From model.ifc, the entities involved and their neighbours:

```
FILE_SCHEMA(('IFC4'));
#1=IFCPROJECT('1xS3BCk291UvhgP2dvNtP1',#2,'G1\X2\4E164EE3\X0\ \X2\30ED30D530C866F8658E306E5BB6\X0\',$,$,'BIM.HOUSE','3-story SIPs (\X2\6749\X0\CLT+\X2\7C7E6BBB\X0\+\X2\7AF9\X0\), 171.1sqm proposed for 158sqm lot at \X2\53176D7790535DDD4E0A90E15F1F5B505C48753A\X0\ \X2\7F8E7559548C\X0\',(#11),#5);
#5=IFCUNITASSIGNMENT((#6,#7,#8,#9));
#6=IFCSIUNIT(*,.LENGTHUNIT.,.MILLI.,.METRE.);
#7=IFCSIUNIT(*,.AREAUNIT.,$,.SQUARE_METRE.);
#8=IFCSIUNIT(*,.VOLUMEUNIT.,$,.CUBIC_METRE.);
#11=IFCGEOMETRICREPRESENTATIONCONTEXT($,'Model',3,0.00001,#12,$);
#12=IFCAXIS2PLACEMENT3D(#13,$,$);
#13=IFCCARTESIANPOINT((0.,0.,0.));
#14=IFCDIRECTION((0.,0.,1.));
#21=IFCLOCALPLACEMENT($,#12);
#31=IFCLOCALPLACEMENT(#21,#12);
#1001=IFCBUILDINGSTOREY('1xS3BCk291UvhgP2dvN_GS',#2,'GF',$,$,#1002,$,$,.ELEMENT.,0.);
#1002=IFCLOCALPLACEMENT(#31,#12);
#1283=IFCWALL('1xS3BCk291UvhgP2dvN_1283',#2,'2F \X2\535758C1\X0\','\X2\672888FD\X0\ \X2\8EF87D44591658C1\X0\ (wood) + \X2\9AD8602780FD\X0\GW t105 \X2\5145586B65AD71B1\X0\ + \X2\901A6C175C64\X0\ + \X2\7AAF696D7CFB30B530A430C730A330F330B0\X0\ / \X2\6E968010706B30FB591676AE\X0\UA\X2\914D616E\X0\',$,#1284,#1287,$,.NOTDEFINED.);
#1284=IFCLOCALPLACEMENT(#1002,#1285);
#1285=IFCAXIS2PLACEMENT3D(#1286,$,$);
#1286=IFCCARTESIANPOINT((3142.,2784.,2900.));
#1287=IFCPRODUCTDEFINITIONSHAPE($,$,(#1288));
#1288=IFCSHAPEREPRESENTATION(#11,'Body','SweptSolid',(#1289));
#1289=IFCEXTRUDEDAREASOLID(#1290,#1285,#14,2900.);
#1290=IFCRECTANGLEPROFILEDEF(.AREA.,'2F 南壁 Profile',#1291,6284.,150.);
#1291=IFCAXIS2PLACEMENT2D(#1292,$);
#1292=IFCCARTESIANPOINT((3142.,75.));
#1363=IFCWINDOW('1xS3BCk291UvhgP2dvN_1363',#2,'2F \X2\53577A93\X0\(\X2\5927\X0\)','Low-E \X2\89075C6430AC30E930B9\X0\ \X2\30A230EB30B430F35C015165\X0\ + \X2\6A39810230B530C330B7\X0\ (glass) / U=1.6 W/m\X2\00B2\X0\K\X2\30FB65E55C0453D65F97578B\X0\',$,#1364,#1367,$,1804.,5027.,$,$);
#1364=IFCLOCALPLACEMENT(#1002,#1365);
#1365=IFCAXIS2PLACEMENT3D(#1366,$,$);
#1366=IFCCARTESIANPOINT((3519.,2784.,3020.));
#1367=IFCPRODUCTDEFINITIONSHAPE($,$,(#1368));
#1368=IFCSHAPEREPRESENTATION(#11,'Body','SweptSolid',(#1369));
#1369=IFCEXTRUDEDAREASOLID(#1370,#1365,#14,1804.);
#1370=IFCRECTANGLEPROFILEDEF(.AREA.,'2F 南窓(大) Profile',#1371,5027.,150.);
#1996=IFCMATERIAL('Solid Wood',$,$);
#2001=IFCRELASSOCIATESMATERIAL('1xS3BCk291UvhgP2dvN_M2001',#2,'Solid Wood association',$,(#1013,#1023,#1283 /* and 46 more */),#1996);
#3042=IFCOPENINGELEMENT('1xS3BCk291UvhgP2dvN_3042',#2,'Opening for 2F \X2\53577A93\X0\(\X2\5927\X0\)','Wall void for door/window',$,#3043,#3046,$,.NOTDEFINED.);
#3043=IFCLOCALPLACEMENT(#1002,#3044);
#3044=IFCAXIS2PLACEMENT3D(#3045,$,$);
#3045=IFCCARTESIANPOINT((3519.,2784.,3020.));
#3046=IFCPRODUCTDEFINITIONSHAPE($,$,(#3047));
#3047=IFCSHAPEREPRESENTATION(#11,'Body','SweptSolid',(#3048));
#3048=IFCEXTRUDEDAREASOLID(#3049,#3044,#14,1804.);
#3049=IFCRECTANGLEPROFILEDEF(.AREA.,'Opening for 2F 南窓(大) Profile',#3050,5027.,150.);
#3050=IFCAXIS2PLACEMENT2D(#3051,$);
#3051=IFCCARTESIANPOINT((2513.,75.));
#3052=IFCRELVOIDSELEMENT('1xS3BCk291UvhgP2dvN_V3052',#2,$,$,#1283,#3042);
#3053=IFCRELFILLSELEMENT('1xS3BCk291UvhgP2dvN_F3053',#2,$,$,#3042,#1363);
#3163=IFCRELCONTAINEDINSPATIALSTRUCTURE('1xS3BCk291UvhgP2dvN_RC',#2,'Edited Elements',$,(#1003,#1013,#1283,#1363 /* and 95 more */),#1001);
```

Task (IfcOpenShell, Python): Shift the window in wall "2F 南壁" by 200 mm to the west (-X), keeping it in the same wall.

```python
import ifcopenshell
import ifcopenshell.api.geometry
import ifcopenshell.util.placement

model = ifcopenshell.open("model.ifc")

window = model.by_guid("1xS3BCk291UvhgP2dvN_1363")
opening = window.FillsVoids[0].RelatingOpeningElement
wall = opening.VoidsElements[0].RelatingBuildingElement

wall_matrix = ifcopenshell.util.placement.get_local_placement(wall.ObjectPlacement)
shift = wall_matrix[:3, 0] * -200.0
before = ifcopenshell.util.placement.get_local_placement(window.ObjectPlacement)[:3, 3].copy()

# The window is not placed relative to its opening, so move both.
for product in (opening, window):
    matrix = ifcopenshell.util.placement.get_local_placement(product.ObjectPlacement)
    matrix[:3, 3] += shift
    ifcopenshell.api.geometry.edit_object_placement(model, product=product, matrix=matrix, is_si=False)

after = ifcopenshell.util.placement.get_local_placement(window.ObjectPlacement)[:3, 3]
print("window moved by", (after - before).round(3) + 0.0)

model.write("model_updated.ifc")
```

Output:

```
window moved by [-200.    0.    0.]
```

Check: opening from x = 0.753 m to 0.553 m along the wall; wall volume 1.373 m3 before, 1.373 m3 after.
